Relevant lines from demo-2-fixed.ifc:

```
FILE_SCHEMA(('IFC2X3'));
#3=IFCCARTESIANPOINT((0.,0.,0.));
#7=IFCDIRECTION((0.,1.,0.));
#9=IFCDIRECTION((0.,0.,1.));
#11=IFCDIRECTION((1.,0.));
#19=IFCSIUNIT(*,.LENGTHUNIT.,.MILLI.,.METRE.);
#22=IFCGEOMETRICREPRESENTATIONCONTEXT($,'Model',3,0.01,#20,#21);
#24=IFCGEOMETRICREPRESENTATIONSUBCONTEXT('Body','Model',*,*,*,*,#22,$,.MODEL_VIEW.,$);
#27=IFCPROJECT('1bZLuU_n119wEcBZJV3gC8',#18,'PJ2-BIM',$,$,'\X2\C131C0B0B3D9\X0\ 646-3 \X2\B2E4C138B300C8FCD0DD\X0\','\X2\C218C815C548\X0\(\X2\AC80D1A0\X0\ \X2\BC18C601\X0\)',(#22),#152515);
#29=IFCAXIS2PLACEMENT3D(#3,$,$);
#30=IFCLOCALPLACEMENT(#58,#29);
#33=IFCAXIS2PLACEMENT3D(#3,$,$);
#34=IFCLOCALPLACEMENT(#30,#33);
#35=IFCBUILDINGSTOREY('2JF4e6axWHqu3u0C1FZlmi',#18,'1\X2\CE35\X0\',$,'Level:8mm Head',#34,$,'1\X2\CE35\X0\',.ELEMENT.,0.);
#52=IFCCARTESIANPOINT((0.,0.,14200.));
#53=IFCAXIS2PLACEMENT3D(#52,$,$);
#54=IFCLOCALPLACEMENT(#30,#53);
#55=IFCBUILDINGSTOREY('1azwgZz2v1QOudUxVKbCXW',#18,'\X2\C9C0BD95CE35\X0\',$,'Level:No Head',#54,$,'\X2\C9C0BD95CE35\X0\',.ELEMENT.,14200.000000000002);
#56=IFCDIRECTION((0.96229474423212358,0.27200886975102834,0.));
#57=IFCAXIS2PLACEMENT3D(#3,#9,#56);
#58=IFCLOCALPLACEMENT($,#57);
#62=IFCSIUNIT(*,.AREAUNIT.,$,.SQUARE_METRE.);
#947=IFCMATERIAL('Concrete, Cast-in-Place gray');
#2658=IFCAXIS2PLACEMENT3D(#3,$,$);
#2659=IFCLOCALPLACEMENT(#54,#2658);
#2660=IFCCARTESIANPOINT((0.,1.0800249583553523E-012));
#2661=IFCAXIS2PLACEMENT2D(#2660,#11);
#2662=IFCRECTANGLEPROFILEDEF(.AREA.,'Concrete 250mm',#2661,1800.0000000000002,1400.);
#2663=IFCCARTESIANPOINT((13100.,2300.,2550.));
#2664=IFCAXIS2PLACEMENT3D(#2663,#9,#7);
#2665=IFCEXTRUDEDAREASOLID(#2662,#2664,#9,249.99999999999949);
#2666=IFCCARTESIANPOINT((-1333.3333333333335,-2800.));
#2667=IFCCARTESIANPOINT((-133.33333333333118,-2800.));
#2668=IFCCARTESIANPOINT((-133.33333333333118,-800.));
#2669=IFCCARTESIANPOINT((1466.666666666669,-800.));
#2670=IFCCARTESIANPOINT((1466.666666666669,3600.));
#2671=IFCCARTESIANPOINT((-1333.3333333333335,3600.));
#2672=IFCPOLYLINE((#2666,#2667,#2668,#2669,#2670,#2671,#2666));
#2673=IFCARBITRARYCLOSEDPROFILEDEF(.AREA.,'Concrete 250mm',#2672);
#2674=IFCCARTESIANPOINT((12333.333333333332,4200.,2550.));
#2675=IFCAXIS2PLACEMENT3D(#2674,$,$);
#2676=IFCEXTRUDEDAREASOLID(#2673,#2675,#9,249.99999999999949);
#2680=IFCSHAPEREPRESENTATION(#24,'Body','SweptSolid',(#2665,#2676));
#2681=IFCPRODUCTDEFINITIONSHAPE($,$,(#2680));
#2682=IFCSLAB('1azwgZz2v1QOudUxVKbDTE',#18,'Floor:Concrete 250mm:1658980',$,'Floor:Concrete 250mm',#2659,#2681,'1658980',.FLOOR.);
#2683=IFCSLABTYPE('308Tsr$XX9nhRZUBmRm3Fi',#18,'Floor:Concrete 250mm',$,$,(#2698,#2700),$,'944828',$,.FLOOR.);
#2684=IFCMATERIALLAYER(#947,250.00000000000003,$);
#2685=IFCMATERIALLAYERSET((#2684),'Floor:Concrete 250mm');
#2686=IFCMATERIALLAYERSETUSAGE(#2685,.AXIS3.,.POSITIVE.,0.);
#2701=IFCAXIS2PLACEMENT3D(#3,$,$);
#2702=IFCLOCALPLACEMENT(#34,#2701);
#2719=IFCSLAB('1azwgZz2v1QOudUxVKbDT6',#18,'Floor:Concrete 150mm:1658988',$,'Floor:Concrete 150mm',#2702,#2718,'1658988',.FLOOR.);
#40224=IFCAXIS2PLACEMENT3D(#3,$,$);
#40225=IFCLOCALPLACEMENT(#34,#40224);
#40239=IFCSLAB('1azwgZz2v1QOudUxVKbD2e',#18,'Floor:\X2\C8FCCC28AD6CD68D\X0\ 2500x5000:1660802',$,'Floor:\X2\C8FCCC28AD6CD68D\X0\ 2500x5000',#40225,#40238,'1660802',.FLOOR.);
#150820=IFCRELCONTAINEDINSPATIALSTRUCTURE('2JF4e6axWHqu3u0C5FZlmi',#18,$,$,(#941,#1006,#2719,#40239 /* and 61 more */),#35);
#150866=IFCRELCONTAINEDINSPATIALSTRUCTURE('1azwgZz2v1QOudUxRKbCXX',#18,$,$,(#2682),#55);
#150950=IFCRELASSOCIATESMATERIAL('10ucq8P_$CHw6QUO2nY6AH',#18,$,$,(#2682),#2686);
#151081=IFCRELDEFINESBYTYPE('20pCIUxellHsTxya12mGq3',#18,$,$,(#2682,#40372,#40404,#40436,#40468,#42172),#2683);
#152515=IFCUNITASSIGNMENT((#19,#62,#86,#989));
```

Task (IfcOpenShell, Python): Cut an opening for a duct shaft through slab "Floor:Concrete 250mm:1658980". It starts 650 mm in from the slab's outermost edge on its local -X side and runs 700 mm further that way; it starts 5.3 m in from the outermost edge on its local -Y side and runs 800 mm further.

```python
import numpy as np
import ifcopenshell
import ifcopenshell.api.feature
import ifcopenshell.api.geometry
import ifcopenshell.api.root
import ifcopenshell.geom
import ifcopenshell.util.placement
import ifcopenshell.util.representation
import ifcopenshell.util.shape
import ifcopenshell.util.unit

model = ifcopenshell.open("demo-2-fixed.ifc")
unit_scale = ifcopenshell.util.unit.calculate_unit_scale(model)
settings = ifcopenshell.geom.settings()


def volume(element):
    """Net volume in cubic metres, openings subtracted."""
    shape = ifcopenshell.geom.create_shape(settings, element)
    return ifcopenshell.util.shape.get_volume(shape.geometry)


slab = model.by_guid("1azwgZz2v1QOudUxVKbDTE")
before = volume(slab)

# Extent in the slab's own axes, in metres. The edges named are its -X and -Y sides.
slab_shape = ifcopenshell.geom.create_shape(settings, slab)
vertices = ifcopenshell.util.shape.get_vertices(slab_shape.geometry)
x_min, y_min, bottom = vertices.min(axis=0)
top = vertices[:, 2].max()

opening = ifcopenshell.api.root.create_entity(model, ifc_class="IfcOpeningElement", name="Duct shaft opening")
context = ifcopenshell.util.representation.get_context(model, "Model", "Body", "MODEL_VIEW")
width, depth = 0.7, 0.8
outline = [(0.0, 0.0), (width, 0.0), (width, depth), (0.0, depth), (0.0, 0.0)]
# Overshoot both faces by 50 mm so the cut is clean.
shape = ifcopenshell.api.geometry.add_slab_representation(
    model, context=context, depth=top - bottom + 0.1, polyline=outline
)
ifcopenshell.api.geometry.assign_representation(model, product=opening, representation=shape)

matrix = ifcopenshell.util.placement.get_local_placement(slab.ObjectPlacement)
matrix[:, 3] = matrix @ np.append(np.array([x_min + 0.65, y_min + 5.3, bottom - 0.05]) / unit_scale, 1.0)
ifcopenshell.api.geometry.edit_object_placement(model, product=opening, matrix=matrix, is_si=False)
ifcopenshell.api.feature.add_feature(model, feature=opening, element=slab)

after = volume(slab)

print(f"slab volume {before:.3f} -> {after:.3f} m3")

model.write("demo-2-fixed_edited.ifc")
```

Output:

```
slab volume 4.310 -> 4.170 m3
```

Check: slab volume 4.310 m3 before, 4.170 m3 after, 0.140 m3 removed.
